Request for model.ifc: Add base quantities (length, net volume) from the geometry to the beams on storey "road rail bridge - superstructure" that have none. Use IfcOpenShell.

First a look at what the model holds.

```python
import ifcopenshell
import ifcopenshell.util.element
import ifcopenshell.util.unit

model = ifcopenshell.open("model.ifc")
print(model.schema)
for unit_type in ("LENGTHUNIT", "AREAUNIT", "VOLUMEUNIT"):
    print(unit_type, ifcopenshell.util.unit.calculate_unit_scale(model, unit_type))
storey = next(s for s in model.by_type("IfcBuildingStorey") if s.Name == "road rail bridge - superstructure")
beams = [e for e in ifcopenshell.util.element.get_decomposition(storey) if e.is_a("IfcBeam")]
for e in sorted(beams, key=lambda e: e.id()):
    print(e.id(), e.is_a(), e.Name, list(ifcopenshell.util.element.get_psets(e, qtos_only=True)), sep=" | ")
```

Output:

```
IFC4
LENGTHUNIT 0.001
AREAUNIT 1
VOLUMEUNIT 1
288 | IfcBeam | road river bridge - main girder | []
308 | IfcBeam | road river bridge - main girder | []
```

```python
import ifcopenshell
import ifcopenshell.api.pset
import ifcopenshell.geom
import ifcopenshell.util.element
import ifcopenshell.util.shape
import ifcopenshell.util.unit

model = ifcopenshell.open("model.ifc")
unit_scale = ifcopenshell.util.unit.calculate_unit_scale(model)
volume_scale = ifcopenshell.util.unit.calculate_unit_scale(model, "VOLUMEUNIT")
settings = ifcopenshell.geom.settings()

storey = next(s for s in model.by_type("IfcBuildingStorey") if s.Name == "road rail bridge - superstructure")
beams = [e for e in ifcopenshell.util.element.get_decomposition(storey) if e.is_a("IfcBeam")]

for e in sorted(beams, key=lambda e: e.id()):
    if ifcopenshell.util.element.get_psets(e, qtos_only=True, should_inherit=False):
        continue
    # Geometry comes back in metres, in the element's own axes.
    shape = ifcopenshell.geom.create_shape(settings, e)
    values = {
        "Length": ifcopenshell.util.shape.get_max_xyz(shape.geometry) / unit_scale,
        "NetVolume": ifcopenshell.util.shape.get_volume(shape.geometry) / volume_scale,
    }
    qto = ifcopenshell.api.pset.add_qto(model, product=e, name="Qto_BeamBaseQuantities")
    ifcopenshell.api.pset.edit_qto(model, qto=qto, properties=values)
    print(e.id(), {k: round(v, 3) for k, v in values.items()})

model.write("model-out.ifc")
```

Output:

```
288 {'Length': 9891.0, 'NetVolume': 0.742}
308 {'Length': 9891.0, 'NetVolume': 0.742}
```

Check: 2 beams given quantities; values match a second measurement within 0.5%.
